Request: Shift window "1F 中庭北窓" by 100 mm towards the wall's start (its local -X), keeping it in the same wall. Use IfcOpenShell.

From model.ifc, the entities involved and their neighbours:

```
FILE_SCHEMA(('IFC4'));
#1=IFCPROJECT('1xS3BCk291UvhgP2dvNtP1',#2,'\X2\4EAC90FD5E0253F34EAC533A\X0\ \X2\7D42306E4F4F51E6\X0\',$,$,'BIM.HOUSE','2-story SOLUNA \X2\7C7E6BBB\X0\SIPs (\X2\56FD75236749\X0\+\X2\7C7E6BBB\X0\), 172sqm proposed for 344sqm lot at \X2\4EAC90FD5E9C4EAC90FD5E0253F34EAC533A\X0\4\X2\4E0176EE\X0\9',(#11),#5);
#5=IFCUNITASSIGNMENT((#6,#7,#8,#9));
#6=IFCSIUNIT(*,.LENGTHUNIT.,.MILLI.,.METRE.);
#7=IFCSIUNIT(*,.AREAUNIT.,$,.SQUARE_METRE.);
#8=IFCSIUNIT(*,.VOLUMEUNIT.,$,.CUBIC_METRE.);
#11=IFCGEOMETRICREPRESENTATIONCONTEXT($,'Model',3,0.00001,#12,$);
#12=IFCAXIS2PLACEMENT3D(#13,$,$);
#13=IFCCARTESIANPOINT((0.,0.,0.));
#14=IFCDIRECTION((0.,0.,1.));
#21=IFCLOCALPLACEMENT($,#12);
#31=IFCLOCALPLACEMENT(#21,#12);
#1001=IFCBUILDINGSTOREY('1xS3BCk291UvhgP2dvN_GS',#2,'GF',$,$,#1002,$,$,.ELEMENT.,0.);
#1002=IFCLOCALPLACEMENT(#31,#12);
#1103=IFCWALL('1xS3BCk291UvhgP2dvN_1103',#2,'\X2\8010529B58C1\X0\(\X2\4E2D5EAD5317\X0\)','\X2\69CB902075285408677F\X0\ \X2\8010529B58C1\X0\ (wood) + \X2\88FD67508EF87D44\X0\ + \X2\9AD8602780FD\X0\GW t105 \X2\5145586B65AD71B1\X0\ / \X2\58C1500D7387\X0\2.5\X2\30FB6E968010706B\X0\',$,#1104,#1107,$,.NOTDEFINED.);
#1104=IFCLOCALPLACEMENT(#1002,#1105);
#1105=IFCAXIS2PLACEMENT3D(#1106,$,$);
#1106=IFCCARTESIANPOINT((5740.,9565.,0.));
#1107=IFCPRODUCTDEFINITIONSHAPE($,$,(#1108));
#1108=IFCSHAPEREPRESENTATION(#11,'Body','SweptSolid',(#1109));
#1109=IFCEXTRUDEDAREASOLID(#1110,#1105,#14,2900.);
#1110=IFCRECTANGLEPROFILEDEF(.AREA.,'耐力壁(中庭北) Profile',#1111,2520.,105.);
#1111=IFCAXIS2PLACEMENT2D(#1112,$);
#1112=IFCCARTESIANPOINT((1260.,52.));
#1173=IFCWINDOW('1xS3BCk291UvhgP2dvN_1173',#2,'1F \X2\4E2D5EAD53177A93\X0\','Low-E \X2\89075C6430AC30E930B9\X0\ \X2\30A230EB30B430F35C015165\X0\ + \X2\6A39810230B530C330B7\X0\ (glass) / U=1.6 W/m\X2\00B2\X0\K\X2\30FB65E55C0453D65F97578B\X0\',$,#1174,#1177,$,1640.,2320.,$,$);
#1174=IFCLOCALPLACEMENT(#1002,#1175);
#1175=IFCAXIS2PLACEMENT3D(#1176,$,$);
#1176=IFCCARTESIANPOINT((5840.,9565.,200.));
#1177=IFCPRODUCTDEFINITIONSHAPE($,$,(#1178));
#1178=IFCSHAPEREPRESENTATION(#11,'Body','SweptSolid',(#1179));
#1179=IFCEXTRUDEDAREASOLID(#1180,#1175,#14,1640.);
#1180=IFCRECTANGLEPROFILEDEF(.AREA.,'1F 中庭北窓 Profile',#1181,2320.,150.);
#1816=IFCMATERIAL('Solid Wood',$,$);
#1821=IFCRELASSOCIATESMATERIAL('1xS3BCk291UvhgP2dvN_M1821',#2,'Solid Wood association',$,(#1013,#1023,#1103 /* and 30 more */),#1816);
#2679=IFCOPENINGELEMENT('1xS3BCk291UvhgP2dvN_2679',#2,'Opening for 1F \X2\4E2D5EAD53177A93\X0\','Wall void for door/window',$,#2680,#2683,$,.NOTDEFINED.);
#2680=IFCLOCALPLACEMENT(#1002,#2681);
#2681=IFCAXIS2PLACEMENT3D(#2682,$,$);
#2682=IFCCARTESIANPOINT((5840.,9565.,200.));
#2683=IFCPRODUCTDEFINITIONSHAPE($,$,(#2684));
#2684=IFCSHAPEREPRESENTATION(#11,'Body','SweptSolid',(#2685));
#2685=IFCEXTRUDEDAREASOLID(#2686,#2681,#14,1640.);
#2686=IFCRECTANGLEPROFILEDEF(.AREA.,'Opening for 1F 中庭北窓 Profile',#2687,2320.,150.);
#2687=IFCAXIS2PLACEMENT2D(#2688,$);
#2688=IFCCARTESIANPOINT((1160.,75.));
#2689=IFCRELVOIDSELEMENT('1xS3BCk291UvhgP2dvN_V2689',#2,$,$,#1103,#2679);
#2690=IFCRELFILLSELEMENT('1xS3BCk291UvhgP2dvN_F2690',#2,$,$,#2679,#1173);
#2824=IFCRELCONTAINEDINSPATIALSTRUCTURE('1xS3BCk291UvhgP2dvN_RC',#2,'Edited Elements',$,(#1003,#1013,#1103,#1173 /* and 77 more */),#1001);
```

```python
import ifcopenshell
import ifcopenshell.api.geometry
import ifcopenshell.util.placement

model = ifcopenshell.open("model.ifc")

window = model.by_guid("1xS3BCk291UvhgP2dvN_1173")
opening = window.FillsVoids[0].RelatingOpeningElement
wall = opening.VoidsElements[0].RelatingBuildingElement

wall_matrix = ifcopenshell.util.placement.get_local_placement(wall.ObjectPlacement)
shift = wall_matrix[:3, 0] * -100.0
before = ifcopenshell.util.placement.get_local_placement(window.ObjectPlacement)[:3, 3].copy()

# The window is not placed relative to its opening, so move both.
for product in (opening, window):
    matrix = ifcopenshell.util.placement.get_local_placement(product.ObjectPlacement)
    matrix[:3, 3] += shift
    ifcopenshell.api.geometry.edit_object_placement(model, product=product, matrix=matrix, is_si=False)

after = ifcopenshell.util.placement.get_local_placement(window.ObjectPlacement)[:3, 3]
print("window moved by", (after - before).round(3) + 0.0)

model.write("model-out.ifc")
```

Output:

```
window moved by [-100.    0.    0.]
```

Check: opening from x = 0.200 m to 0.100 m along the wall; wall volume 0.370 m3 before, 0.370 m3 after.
